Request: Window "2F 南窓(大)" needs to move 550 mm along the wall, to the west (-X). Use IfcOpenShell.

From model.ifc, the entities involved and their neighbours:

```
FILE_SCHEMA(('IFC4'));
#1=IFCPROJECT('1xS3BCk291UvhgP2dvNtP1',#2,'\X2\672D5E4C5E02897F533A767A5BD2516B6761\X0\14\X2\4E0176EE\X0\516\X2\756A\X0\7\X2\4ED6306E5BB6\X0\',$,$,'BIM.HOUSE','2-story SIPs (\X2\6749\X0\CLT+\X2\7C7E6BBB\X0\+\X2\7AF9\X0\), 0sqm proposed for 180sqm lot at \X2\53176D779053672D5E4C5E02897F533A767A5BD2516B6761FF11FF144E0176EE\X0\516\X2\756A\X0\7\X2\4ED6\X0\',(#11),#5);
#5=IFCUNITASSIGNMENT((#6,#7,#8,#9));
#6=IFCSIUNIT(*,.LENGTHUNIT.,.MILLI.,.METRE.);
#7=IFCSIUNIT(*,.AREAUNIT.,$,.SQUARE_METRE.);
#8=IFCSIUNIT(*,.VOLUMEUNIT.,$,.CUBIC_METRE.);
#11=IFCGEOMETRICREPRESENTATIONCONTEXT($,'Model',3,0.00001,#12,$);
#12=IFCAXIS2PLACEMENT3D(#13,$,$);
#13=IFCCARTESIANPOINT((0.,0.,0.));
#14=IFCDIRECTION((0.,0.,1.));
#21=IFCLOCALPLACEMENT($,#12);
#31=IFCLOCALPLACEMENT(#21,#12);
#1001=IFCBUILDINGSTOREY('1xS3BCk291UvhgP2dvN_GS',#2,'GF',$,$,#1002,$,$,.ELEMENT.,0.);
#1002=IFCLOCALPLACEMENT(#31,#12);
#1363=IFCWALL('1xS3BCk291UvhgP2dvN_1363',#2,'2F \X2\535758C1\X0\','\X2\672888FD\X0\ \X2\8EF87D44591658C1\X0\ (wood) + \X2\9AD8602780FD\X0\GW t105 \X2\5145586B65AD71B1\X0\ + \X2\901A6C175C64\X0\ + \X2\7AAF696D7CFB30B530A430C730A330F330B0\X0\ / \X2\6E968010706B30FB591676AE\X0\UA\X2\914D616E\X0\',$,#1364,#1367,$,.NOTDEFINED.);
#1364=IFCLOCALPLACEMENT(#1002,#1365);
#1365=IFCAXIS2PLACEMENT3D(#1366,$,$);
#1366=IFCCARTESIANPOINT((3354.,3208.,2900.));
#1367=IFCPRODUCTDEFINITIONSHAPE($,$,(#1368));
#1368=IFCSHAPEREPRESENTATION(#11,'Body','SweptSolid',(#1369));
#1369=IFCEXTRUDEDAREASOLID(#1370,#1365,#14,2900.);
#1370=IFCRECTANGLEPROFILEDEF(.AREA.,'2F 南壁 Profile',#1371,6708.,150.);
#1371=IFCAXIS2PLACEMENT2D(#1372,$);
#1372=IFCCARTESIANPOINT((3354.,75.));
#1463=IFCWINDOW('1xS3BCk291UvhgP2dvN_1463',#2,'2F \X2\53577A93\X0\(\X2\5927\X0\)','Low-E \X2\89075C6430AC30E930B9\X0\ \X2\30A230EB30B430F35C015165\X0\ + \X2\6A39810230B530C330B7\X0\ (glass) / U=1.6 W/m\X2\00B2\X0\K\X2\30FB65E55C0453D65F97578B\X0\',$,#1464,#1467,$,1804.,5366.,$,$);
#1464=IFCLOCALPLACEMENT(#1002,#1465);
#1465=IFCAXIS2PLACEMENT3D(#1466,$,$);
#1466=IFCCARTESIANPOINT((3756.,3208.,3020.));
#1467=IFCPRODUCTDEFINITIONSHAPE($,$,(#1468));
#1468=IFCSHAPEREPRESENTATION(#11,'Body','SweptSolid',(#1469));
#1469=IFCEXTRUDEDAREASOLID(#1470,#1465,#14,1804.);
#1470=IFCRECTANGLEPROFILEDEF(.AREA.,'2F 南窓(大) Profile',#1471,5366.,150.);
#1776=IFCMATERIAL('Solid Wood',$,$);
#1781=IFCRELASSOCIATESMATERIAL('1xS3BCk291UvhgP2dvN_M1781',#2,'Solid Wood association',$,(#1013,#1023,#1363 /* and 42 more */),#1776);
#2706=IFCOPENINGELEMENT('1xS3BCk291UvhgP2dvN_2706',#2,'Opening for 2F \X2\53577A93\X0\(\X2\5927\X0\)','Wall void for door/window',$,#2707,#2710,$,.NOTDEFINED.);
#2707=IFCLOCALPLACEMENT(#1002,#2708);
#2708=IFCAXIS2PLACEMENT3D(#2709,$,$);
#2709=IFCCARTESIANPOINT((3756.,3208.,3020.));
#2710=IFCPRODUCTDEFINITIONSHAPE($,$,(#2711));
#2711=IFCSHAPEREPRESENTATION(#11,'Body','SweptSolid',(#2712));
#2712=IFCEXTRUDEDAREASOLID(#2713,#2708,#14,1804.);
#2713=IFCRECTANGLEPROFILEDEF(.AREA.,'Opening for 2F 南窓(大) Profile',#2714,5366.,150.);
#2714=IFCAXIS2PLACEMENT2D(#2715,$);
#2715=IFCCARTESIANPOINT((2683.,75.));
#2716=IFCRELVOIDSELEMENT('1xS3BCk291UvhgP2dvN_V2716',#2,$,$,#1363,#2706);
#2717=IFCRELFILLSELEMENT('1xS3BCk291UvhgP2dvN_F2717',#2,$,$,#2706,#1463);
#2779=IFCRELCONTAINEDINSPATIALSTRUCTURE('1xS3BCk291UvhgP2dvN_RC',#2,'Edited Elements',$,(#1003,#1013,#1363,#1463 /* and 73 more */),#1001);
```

```python
import ifcopenshell
import ifcopenshell.api.geometry
import ifcopenshell.util.placement

model = ifcopenshell.open("model.ifc")

window = model.by_guid("1xS3BCk291UvhgP2dvN_1463")
opening = window.FillsVoids[0].RelatingOpeningElement
wall = opening.VoidsElements[0].RelatingBuildingElement

wall_matrix = ifcopenshell.util.placement.get_local_placement(wall.ObjectPlacement)
shift = wall_matrix[:3, 0] * -550.0
before = ifcopenshell.util.placement.get_local_placement(window.ObjectPlacement)[:3, 3].copy()

# The window is not placed relative to its opening, so move both.
for product in (opening, window):
    matrix = ifcopenshell.util.placement.get_local_placement(product.ObjectPlacement)
    matrix[:3, 3] += shift
    ifcopenshell.api.geometry.edit_object_placement(model, product=product, matrix=matrix, is_si=False)

after = ifcopenshell.util.placement.get_local_placement(window.ObjectPlacement)[:3, 3]
print("window moved by", (after - before).round(3) + 0.0)

model.write("model_rev.ifc")
```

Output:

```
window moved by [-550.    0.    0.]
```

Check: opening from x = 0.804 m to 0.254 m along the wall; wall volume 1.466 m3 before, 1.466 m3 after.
